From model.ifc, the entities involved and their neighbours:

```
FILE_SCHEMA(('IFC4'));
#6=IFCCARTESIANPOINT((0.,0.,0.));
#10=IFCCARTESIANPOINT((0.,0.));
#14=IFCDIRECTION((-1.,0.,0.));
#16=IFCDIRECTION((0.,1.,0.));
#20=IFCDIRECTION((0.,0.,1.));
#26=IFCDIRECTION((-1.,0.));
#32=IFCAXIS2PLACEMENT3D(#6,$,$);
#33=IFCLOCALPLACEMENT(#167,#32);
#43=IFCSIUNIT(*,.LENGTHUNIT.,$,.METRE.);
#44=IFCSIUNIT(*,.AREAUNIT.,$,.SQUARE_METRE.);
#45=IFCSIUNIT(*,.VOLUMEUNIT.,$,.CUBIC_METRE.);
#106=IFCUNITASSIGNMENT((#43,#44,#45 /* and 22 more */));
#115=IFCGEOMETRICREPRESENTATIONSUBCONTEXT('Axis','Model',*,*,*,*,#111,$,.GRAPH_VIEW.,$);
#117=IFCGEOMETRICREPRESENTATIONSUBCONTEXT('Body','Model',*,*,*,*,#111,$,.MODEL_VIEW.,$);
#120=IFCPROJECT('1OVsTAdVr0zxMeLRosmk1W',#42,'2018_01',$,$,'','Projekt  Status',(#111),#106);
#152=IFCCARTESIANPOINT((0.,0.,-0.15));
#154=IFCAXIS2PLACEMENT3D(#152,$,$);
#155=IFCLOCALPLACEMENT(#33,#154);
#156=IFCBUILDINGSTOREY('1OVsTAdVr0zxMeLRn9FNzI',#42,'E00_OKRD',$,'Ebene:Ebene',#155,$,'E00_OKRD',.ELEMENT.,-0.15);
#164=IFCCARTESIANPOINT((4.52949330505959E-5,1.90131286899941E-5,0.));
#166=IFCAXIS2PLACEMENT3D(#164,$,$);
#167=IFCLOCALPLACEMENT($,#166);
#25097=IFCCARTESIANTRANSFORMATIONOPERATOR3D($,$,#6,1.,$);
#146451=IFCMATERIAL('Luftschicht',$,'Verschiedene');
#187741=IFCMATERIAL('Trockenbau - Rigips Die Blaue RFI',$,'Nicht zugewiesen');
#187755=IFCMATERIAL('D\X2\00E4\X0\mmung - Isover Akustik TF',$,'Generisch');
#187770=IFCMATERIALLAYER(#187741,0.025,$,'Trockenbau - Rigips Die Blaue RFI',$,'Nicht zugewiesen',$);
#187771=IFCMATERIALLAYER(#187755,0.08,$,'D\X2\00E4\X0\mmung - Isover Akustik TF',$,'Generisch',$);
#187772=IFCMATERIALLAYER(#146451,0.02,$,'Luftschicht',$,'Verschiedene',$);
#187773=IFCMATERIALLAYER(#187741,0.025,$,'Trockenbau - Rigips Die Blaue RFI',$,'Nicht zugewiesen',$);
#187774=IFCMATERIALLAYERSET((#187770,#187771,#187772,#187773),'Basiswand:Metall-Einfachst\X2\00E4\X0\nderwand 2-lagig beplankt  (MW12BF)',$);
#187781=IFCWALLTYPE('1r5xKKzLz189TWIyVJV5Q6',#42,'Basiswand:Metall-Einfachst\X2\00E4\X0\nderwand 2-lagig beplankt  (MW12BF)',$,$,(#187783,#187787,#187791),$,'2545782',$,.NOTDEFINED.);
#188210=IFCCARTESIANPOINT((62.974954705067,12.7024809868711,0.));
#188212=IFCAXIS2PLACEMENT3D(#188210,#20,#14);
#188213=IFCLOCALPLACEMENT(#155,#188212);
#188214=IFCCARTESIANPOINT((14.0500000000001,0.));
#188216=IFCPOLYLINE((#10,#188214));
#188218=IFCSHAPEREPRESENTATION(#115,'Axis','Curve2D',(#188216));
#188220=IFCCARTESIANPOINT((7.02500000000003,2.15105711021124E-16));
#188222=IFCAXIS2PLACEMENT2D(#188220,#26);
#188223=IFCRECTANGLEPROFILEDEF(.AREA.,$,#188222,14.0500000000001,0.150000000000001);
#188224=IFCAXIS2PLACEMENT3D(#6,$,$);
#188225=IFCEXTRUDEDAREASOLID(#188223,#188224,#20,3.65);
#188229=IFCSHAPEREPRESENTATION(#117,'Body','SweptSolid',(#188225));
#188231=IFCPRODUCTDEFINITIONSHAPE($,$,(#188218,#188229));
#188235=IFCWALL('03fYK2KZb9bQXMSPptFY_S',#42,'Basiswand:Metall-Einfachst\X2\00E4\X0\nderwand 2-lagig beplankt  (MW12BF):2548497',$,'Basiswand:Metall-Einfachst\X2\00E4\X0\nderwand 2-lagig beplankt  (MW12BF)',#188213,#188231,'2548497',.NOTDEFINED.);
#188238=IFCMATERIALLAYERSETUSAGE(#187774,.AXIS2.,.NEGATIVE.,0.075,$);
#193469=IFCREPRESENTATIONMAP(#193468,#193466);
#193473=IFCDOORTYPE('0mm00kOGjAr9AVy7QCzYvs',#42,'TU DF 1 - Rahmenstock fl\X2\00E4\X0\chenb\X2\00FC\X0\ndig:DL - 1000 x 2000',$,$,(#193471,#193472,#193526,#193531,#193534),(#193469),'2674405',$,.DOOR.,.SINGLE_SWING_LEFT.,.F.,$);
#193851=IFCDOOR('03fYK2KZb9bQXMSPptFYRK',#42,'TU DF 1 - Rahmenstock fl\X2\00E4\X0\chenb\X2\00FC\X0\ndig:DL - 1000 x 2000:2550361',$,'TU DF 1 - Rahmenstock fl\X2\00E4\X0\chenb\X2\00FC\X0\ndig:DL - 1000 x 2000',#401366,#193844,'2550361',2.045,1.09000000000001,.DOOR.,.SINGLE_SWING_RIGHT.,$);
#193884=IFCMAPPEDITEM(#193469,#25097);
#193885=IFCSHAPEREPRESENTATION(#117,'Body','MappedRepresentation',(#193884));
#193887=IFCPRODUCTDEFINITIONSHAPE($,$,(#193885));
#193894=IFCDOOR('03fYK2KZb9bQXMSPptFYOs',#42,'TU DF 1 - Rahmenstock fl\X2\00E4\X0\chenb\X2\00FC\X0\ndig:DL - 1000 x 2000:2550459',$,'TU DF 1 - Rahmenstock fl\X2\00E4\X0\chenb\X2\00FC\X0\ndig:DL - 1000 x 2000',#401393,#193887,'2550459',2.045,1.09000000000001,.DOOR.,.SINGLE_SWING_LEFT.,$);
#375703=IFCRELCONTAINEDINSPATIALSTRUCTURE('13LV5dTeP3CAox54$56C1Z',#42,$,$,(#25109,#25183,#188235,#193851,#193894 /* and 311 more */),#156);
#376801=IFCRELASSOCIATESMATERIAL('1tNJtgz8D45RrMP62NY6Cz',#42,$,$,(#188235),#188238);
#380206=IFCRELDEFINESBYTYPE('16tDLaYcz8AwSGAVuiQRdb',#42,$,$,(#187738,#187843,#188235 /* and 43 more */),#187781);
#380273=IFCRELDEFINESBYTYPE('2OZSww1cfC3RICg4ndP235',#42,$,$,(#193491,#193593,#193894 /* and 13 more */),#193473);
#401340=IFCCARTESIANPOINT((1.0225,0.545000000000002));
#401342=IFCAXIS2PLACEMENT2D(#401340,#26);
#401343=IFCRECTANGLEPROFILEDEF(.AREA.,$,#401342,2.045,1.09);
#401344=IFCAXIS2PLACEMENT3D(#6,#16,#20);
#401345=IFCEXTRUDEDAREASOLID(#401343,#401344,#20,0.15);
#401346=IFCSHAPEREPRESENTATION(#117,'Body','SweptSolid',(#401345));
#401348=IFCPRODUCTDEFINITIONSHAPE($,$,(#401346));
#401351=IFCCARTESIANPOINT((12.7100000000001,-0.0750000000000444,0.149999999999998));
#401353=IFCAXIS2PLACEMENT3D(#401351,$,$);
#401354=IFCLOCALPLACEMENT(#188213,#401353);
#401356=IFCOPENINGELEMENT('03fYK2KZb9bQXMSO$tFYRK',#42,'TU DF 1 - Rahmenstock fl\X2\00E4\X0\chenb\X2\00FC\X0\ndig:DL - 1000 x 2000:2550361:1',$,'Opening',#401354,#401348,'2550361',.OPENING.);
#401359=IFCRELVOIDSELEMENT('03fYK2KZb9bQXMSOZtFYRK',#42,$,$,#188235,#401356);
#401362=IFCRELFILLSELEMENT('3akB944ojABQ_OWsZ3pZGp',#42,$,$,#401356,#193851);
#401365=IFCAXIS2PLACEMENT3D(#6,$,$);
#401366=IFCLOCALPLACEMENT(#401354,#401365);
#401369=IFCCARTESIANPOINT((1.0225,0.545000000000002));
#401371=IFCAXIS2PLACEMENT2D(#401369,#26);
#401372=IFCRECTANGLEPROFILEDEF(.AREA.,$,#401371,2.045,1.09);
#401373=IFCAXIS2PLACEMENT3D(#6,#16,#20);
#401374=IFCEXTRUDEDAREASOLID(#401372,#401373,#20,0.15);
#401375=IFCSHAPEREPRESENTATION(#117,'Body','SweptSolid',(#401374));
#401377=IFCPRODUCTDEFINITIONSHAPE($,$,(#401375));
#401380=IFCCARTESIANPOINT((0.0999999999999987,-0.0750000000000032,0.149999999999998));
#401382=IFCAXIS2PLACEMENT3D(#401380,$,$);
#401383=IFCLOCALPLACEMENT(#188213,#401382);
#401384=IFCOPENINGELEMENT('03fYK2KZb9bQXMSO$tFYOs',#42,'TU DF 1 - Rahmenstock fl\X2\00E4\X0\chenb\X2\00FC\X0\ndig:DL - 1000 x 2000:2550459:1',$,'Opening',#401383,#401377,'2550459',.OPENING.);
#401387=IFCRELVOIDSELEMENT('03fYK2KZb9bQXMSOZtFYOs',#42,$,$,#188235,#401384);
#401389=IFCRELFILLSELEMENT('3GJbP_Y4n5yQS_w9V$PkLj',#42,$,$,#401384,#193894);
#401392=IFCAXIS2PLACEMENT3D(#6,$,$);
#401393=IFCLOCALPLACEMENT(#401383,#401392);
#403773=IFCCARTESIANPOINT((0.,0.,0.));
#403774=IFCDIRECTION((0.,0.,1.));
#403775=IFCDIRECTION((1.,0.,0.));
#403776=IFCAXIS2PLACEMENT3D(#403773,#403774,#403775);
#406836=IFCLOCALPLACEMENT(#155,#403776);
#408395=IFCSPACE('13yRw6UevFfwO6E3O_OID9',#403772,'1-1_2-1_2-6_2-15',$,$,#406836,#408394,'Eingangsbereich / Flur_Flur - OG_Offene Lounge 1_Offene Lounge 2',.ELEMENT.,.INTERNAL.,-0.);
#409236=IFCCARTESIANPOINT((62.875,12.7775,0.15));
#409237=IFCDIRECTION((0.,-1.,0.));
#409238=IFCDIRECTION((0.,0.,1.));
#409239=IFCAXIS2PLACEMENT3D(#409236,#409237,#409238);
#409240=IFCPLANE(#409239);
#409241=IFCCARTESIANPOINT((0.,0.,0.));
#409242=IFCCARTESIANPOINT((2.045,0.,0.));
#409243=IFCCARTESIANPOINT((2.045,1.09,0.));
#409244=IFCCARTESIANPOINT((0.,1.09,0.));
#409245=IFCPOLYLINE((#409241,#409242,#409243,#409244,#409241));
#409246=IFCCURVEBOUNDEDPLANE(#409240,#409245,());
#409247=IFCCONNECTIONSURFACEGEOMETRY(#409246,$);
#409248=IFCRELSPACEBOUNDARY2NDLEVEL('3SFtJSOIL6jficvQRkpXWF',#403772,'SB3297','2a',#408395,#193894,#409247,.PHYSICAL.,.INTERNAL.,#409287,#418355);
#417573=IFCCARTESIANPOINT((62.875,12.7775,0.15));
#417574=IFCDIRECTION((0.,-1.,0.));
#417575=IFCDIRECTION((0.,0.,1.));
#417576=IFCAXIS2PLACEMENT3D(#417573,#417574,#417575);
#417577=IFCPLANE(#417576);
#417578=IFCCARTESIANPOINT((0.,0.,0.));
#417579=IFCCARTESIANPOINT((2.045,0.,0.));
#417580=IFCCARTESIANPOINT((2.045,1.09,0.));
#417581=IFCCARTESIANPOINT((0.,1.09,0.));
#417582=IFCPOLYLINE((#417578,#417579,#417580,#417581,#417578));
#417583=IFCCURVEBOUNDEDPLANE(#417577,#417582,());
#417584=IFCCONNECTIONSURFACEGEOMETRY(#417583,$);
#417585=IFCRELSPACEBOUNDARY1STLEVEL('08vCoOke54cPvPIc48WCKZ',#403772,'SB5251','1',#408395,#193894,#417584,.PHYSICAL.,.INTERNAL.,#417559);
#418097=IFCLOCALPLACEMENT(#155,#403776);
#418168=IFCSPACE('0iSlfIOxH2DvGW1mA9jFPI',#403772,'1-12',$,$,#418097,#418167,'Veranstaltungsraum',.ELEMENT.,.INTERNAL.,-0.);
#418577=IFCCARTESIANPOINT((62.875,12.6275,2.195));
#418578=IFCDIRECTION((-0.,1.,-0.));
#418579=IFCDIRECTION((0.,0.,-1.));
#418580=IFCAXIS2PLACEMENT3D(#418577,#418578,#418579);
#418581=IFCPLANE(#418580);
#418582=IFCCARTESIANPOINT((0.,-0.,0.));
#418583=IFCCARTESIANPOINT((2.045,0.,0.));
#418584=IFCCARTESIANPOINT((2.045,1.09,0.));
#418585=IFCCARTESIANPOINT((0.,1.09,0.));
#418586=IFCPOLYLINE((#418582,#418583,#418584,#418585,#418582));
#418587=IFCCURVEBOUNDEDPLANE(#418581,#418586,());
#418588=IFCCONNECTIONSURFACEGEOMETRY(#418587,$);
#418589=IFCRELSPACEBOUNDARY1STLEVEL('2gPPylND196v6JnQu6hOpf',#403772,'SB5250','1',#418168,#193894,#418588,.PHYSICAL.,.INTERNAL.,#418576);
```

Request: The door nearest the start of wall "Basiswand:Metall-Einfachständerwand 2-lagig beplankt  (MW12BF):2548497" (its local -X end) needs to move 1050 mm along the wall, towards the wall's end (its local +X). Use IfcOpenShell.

```python
import numpy as np
import ifcopenshell
import ifcopenshell.api.geometry
import ifcopenshell.util.placement
import ifcopenshell.util.unit

model = ifcopenshell.open("model.ifc")
unit_scale = ifcopenshell.util.unit.calculate_unit_scale(model)

door = model.by_id(193894)
opening = door.FillsVoids[0].RelatingOpeningElement
wall = opening.VoidsElements[0].RelatingBuildingElement

wall_matrix = ifcopenshell.util.placement.get_local_placement(wall.ObjectPlacement)
shift = wall_matrix[:3, 0] * 1.05 / unit_scale
before = ifcopenshell.util.placement.get_local_placement(door.ObjectPlacement)[:3, 3].copy()

# The door is placed relative to its opening, so it follows when the opening moves.
matrix = ifcopenshell.util.placement.get_local_placement(opening.ObjectPlacement)
matrix[:3, 3] += shift
ifcopenshell.api.geometry.edit_object_placement(
    model, product=opening, matrix=matrix, is_si=False, should_transform_children=True
)

# Space boundary surfaces are stored in each space's coordinates; move them too.
for rel in door.ProvidesBoundaries:
    if not rel.ConnectionGeometry:
        continue
    surface = rel.ConnectionGeometry.SurfaceOnRelatingElement.BasisSurface
    space_matrix = ifcopenshell.util.placement.get_local_placement(rel.RelatingSpace.ObjectPlacement)
    point = np.array(surface.Position.Location.Coordinates) + space_matrix[:3, :3].T @ shift
    surface.Position = model.createIfcAxis2Placement3D(
        model.createIfcCartesianPoint(point.tolist()), surface.Position.Axis, surface.Position.RefDirection
    )

after = ifcopenshell.util.placement.get_local_placement(door.ObjectPlacement)[:3, 3]
print("door moved by", (after - before).round(3) + 0.0)

model.write("model_edited.ifc")
```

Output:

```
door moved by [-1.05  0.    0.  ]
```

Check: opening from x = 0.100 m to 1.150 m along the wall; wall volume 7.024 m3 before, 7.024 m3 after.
